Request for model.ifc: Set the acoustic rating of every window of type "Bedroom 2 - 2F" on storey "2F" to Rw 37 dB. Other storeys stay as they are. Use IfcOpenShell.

First a look at what the model holds.

```python
import ifcopenshell
import ifcopenshell.util.element

model = ifcopenshell.open("model.ifc")
print(model.schema)
storey = next(s for s in model.by_type("IfcBuildingStorey") if s.Name == "2F")
windows = [e for e in ifcopenshell.util.element.get_decomposition(storey) if e.is_a("IfcWindow")]
seen = {}
for e in windows:
    element_type = ifcopenshell.util.element.get_type(e)
    key = (element_type.Name if element_type != e and element_type else None, ifcopenshell.util.element.get_pset(e, "Pset_WindowCommon", "AcousticRating"))
    seen[key] = seen.get(key, 0) + 1
for (name, value), count in sorted(seen.items(), key=str):
    print(count, "x", name, "|", value)
```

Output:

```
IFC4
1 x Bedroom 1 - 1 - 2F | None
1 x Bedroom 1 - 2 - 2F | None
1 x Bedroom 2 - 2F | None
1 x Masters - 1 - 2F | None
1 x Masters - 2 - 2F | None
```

```python
import ifcopenshell
import ifcopenshell.api.pset
import ifcopenshell.util.element

model = ifcopenshell.open("model.ifc")

storey = next(s for s in model.by_type("IfcBuildingStorey") if s.Name == "2F")
windows = [e for e in ifcopenshell.util.element.get_decomposition(storey) if e.is_a("IfcWindow")]

count = 0
for e in windows:
    element_type = ifcopenshell.util.element.get_type(e)
    if element_type in (None, e) or element_type.Name != "Bedroom 2 - 2F":
        continue
    # add_pset returns the element's existing set when there is one.
    pset = ifcopenshell.api.pset.add_pset(model, product=e, name="Pset_WindowCommon")
    ifcopenshell.api.pset.edit_pset(model, pset=pset, properties={"AcousticRating": "Rw 37 dB"})
    count += 1

print(count, "windows updated")

model.write("model_edited.ifc")
```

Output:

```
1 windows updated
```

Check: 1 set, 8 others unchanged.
